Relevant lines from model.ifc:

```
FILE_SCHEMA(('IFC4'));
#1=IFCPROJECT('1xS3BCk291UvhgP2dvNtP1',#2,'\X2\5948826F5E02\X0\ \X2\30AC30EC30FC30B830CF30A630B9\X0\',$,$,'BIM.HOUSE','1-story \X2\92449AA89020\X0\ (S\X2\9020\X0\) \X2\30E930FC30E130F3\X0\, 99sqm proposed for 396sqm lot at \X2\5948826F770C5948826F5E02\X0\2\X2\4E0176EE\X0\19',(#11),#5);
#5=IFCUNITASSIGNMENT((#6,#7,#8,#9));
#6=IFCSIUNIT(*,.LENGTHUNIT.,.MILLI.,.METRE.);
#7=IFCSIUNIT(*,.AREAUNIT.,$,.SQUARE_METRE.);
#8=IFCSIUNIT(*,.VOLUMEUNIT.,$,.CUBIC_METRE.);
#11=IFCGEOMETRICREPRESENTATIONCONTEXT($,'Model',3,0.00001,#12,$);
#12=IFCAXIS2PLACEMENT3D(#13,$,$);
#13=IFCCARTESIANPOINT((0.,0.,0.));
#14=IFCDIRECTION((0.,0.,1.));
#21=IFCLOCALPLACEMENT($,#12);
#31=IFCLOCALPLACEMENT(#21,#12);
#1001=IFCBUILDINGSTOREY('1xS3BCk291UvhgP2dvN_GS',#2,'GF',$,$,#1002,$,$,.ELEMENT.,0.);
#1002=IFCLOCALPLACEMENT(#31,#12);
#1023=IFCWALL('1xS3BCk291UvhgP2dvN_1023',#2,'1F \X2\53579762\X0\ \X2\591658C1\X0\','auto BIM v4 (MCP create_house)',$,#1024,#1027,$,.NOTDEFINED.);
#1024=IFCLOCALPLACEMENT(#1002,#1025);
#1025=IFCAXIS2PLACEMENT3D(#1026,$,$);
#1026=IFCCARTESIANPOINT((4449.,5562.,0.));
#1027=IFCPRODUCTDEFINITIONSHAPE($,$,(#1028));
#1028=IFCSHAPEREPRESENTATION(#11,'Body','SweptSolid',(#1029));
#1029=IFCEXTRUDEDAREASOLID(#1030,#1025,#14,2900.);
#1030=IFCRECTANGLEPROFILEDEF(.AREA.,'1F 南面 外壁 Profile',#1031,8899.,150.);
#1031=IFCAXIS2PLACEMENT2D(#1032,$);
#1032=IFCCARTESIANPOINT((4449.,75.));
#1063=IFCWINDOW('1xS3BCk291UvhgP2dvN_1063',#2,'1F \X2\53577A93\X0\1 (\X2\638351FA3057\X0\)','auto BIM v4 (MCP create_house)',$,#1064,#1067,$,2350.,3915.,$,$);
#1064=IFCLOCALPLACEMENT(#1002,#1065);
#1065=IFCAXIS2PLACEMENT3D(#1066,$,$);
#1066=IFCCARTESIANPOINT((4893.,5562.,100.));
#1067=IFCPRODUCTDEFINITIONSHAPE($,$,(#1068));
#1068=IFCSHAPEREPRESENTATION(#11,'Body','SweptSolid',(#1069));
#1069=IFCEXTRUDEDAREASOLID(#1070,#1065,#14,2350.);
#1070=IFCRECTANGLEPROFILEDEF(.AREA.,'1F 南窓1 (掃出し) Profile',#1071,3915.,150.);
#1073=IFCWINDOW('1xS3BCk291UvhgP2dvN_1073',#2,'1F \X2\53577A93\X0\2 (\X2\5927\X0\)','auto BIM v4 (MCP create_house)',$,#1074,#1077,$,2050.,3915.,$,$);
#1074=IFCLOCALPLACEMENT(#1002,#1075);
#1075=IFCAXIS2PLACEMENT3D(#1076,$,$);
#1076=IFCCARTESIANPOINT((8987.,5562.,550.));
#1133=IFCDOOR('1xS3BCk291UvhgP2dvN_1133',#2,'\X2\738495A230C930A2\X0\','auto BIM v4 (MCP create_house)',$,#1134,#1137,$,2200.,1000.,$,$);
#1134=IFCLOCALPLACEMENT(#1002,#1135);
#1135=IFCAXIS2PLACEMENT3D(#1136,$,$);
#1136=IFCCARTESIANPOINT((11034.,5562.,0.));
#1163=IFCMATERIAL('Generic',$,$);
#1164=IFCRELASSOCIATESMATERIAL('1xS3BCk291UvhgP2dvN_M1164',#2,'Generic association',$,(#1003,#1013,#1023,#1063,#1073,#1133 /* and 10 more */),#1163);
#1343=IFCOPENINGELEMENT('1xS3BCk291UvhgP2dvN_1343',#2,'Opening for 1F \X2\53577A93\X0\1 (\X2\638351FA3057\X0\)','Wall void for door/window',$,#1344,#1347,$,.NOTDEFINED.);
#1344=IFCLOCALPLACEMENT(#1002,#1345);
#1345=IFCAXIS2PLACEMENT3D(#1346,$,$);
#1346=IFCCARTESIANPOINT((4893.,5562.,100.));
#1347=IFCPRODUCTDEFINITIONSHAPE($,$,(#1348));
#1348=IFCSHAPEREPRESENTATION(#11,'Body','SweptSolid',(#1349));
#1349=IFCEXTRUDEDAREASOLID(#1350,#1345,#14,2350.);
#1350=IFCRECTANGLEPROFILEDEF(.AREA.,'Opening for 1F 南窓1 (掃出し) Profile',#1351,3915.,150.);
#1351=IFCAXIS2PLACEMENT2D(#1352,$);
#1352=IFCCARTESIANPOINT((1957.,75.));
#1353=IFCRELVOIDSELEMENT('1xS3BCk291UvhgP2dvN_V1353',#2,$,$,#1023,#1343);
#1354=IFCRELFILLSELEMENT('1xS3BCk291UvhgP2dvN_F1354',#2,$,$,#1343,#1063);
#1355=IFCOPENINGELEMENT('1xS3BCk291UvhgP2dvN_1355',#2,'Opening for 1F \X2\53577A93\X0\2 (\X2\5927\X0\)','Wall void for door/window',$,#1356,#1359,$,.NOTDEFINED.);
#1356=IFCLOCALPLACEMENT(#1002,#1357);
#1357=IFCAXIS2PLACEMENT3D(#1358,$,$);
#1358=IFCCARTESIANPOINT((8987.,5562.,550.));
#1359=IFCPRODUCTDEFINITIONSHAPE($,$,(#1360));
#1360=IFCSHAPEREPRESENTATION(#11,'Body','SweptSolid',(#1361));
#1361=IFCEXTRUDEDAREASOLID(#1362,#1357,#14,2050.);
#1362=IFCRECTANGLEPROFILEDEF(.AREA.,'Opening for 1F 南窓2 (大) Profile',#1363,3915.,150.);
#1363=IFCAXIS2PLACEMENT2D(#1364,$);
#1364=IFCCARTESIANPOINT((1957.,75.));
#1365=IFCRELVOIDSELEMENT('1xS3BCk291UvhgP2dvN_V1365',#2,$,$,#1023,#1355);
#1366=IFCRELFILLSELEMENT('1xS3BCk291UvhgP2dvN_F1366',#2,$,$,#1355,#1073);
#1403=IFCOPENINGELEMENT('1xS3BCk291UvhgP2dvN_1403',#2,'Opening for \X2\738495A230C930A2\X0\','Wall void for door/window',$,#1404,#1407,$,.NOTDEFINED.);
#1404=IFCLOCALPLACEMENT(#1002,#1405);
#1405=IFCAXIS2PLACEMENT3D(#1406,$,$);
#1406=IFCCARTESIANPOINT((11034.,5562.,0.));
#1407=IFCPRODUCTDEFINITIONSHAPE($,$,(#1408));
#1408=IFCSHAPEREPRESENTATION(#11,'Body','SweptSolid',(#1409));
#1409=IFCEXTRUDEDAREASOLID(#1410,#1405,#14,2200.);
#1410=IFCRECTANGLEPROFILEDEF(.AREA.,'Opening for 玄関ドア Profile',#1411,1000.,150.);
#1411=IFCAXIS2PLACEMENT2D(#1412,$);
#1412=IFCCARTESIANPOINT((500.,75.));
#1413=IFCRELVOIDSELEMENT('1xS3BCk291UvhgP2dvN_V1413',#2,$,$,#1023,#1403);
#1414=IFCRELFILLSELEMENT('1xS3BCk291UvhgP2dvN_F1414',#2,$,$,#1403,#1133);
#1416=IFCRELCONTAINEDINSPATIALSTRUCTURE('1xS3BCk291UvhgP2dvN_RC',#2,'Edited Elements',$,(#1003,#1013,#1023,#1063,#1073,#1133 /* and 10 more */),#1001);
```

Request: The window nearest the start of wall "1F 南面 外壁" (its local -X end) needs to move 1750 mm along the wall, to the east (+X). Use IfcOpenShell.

```python
import ifcopenshell
import ifcopenshell.api.geometry
import ifcopenshell.util.placement

model = ifcopenshell.open("model.ifc")

window = model.by_guid("1xS3BCk291UvhgP2dvN_1063")
opening = window.FillsVoids[0].RelatingOpeningElement
wall = opening.VoidsElements[0].RelatingBuildingElement

wall_matrix = ifcopenshell.util.placement.get_local_placement(wall.ObjectPlacement)
shift = wall_matrix[:3, 0] * 1750.0
before = ifcopenshell.util.placement.get_local_placement(window.ObjectPlacement)[:3, 3].copy()

# The window is not placed relative to its opening, so move both.
for product in (opening, window):
    matrix = ifcopenshell.util.placement.get_local_placement(product.ObjectPlacement)
    matrix[:3, 3] += shift
    ifcopenshell.api.geometry.edit_object_placement(model, product=product, matrix=matrix, is_si=False)

after = ifcopenshell.util.placement.get_local_placement(window.ObjectPlacement)[:3, 3]
print("window moved by", (after - before).round(3) + 0.0)

model.write("model_updated.ifc")
```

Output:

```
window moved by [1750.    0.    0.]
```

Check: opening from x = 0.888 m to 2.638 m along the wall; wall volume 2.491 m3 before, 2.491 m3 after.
